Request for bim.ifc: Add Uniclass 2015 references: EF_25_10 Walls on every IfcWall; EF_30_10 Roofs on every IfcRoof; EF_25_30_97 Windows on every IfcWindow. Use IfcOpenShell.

First a look at what the model holds.

```python
import ifcopenshell

model = ifcopenshell.open("bim.ifc")
print(model.schema)
print("classifications:", [c.Name for c in model.by_type("IfcClassification")])
for ifc_class in ("IfcDoor", "IfcRoof", "IfcStair", "IfcWall", "IfcWindow"):
    print(ifc_class, len(model.by_type(ifc_class)))
```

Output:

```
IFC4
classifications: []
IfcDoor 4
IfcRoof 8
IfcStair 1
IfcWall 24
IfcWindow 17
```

```python
import ifcopenshell
import ifcopenshell.api.classification

model = ifcopenshell.open("bim.ifc")

system = ifcopenshell.api.classification.add_classification(model, classification="Uniclass 2015")

codes = {
    "IfcWall": ("EF_25_10", "Walls"),
    "IfcRoof": ("EF_30_10", "Roofs"),
    "IfcWindow": ("EF_25_30_97", "Windows"),
}
for ifc_class, (code, name) in codes.items():
    products = model.by_type(ifc_class)
    ifcopenshell.api.classification.add_reference(
        model, products=products, classification=system, identification=code, name=name
    )
    print(code, len(products))

model.write("bim-out.ifc")
```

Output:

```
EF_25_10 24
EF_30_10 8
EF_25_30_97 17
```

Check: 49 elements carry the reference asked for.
